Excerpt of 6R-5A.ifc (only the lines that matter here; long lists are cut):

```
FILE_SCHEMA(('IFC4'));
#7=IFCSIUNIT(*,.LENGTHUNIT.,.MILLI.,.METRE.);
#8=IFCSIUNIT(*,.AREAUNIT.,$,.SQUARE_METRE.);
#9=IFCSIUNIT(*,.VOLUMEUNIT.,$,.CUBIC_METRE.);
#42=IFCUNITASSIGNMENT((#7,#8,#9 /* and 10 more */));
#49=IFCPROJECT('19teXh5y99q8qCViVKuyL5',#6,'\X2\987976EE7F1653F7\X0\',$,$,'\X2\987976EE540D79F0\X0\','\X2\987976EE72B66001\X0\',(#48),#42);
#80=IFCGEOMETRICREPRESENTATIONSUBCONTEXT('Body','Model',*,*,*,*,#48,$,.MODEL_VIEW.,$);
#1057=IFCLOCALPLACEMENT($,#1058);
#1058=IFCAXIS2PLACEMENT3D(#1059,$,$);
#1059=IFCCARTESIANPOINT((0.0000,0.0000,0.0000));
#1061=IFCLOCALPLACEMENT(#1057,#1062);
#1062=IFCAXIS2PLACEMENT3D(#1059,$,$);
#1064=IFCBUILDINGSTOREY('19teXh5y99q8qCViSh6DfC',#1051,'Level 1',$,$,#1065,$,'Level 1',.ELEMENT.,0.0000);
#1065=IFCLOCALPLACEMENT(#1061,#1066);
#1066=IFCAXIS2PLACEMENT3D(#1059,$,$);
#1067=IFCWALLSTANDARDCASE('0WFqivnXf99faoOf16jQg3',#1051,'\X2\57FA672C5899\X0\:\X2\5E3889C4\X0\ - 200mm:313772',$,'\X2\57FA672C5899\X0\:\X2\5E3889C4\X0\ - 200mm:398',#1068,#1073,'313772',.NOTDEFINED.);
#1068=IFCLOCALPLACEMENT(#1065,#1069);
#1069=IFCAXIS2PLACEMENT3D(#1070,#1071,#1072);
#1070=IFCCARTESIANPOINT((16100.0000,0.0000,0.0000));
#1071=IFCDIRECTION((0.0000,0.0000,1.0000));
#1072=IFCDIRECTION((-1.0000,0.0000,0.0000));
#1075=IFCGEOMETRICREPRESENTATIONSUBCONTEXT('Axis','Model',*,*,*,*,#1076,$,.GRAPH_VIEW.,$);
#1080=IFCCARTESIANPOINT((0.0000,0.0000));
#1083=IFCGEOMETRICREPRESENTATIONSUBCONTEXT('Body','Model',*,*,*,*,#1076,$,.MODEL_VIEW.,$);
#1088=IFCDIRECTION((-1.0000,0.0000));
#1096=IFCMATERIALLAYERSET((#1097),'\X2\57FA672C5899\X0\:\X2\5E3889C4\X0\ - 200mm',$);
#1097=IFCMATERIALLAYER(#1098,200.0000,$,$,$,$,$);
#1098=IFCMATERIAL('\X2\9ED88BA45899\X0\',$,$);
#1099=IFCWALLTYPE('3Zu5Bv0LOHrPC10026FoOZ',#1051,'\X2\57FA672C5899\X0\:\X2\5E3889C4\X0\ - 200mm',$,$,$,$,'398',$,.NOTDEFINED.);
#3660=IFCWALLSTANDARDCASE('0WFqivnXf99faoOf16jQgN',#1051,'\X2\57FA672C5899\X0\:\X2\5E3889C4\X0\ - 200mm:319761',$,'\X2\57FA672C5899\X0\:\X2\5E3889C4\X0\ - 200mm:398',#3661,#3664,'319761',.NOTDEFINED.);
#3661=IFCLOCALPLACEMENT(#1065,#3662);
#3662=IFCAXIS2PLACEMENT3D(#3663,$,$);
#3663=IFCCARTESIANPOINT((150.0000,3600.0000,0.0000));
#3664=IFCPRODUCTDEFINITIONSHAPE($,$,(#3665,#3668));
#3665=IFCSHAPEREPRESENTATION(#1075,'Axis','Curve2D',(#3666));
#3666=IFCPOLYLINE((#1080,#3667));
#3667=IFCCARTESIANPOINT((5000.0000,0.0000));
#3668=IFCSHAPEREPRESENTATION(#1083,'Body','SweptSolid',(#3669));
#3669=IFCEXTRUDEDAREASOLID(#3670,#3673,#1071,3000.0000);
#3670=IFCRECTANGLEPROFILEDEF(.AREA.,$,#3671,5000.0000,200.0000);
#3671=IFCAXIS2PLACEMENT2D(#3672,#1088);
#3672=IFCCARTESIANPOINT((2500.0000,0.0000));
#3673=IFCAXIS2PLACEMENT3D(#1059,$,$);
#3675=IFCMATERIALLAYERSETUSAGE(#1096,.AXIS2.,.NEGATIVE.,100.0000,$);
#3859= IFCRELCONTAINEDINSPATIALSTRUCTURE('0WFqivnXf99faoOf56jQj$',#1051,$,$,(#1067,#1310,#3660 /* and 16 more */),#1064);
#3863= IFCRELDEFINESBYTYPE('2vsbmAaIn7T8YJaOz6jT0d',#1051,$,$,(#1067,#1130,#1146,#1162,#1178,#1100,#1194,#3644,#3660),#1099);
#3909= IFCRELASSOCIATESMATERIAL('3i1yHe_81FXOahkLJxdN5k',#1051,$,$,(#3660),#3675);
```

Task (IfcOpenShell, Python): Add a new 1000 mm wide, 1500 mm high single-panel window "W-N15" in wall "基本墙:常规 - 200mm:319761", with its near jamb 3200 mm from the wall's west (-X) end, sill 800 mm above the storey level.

```python
import numpy as np
import ifcopenshell
import ifcopenshell.api.feature
import ifcopenshell.api.geometry
import ifcopenshell.api.root
import ifcopenshell.api.spatial
import ifcopenshell.geom
import ifcopenshell.util.element
import ifcopenshell.util.placement
import ifcopenshell.util.representation
import ifcopenshell.util.shape
import ifcopenshell.util.unit

model = ifcopenshell.open("6R-5A.ifc")
unit_scale = ifcopenshell.util.unit.calculate_unit_scale(model)
settings = ifcopenshell.geom.settings()


def volume(element):
    """Net volume in cubic metres, openings subtracted."""
    shape = ifcopenshell.geom.create_shape(settings, element)
    return ifcopenshell.util.shape.get_volume(shape.geometry)


wall = model.by_guid("0WFqivnXf99faoOf16jQgN")
storey = ifcopenshell.util.element.get_container(wall, ifc_class="IfcBuildingStorey")
context = ifcopenshell.util.representation.get_context(model, "Model", "Body", "MODEL_VIEW")
before = volume(wall)

width, height, from_end, sill = 1, 1.5, 3.2, 0.8  # metres

# The wall runs along its own X axis, and the end named is its -X end.
wall_shape = ifcopenshell.geom.create_shape(settings, wall)
x, y, z = ifcopenshell.util.shape.get_vertices(wall_shape.geometry).T
start = x.min() + from_end
face, thickness = float(y.min()), float(y.max() - y.min())
wall_matrix = ifcopenshell.util.placement.get_local_placement(wall.ObjectPlacement)
level = ifcopenshell.util.placement.get_local_placement(storey.ObjectPlacement)[2, 3]


def in_wall(x, y):
    """Placement at x, y metres in the wall's axes, at sill height."""
    matrix = wall_matrix.copy()
    matrix[:, 3] = wall_matrix @ np.array([x / unit_scale, y / unit_scale, 0.0, 1.0])
    matrix[2, 3] = level + sill / unit_scale
    return matrix


# Opening: a box that overshoots both wall faces by 50 mm.
opening = ifcopenshell.api.root.create_entity(model, ifc_class="IfcOpeningElement", predefined_type="OPENING")
box = ifcopenshell.api.geometry.add_wall_representation(
    model, context=context, length=width, height=height, thickness=thickness + 0.1
)
ifcopenshell.api.geometry.assign_representation(model, product=opening, representation=box)
ifcopenshell.api.geometry.edit_object_placement(model, product=opening, matrix=in_wall(start, face - 0.05), is_si=False)
ifcopenshell.api.feature.add_feature(model, feature=opening, element=wall)

window = ifcopenshell.api.root.create_entity(model, ifc_class="IfcWindow", name="W-N15", predefined_type="WINDOW")
window.OverallWidth, window.OverallHeight = width / unit_scale, height / unit_scale
window.PartitioningType = "SINGLE_PANEL"
body = ifcopenshell.api.geometry.add_window_representation(
    model,
    context=context,
    overall_width=window.OverallWidth,
    overall_height=window.OverallHeight,
    partition_type="SINGLE_PANEL",
)
ifcopenshell.api.geometry.assign_representation(model, product=window, representation=body)
ifcopenshell.api.spatial.assign_container(model, products=[window], relating_structure=storey)
ifcopenshell.api.feature.add_filling(model, opening=opening, element=window)

# Centre the window in the wall's thickness.
ifcopenshell.api.geometry.edit_object_placement(model, product=window, matrix=in_wall(start, face), is_si=False)
window_shape = ifcopenshell.geom.create_shape(settings, window)
depth = ifcopenshell.util.shape.get_vertices(window_shape.geometry)[:, 1]
offset = face + thickness / 2 - (depth.min() + depth.max()) / 2
ifcopenshell.api.geometry.edit_object_placement(model, product=window, matrix=in_wall(start, offset), is_si=False)

after = volume(wall)

print(f"wall volume {before:.3f} -> {after:.3f} m3")

model.write("6R-5A_edited.ifc")
```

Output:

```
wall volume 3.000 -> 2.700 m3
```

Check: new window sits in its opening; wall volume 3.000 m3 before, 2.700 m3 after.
